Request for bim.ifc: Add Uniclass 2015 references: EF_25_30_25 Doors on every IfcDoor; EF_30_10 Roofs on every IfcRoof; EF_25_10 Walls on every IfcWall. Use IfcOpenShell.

First a look at what the model holds.

```python
import ifcopenshell

model = ifcopenshell.open("bim.ifc")
print(model.schema)
print("classifications:", [c.Name for c in model.by_type("IfcClassification")])
for ifc_class in ("IfcDoor", "IfcRoof", "IfcStair", "IfcWall", "IfcWindow"):
    print(ifc_class, len(model.by_type(ifc_class)))
```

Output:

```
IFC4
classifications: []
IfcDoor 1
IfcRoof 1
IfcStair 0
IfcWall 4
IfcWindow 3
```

```python
import ifcopenshell
import ifcopenshell.api.classification

model = ifcopenshell.open("bim.ifc")

system = ifcopenshell.api.classification.add_classification(model, classification="Uniclass 2015")

codes = {
    "IfcDoor": ("EF_25_30_25", "Doors"),
    "IfcRoof": ("EF_30_10", "Roofs"),
    "IfcWall": ("EF_25_10", "Walls"),
}
for ifc_class, (code, name) in codes.items():
    products = model.by_type(ifc_class)
    ifcopenshell.api.classification.add_reference(
        model, products=products, classification=system, identification=code, name=name
    )
    print(code, len(products))

model.write("bim_edited.ifc")
```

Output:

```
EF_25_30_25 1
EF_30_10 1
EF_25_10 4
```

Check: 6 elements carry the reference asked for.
